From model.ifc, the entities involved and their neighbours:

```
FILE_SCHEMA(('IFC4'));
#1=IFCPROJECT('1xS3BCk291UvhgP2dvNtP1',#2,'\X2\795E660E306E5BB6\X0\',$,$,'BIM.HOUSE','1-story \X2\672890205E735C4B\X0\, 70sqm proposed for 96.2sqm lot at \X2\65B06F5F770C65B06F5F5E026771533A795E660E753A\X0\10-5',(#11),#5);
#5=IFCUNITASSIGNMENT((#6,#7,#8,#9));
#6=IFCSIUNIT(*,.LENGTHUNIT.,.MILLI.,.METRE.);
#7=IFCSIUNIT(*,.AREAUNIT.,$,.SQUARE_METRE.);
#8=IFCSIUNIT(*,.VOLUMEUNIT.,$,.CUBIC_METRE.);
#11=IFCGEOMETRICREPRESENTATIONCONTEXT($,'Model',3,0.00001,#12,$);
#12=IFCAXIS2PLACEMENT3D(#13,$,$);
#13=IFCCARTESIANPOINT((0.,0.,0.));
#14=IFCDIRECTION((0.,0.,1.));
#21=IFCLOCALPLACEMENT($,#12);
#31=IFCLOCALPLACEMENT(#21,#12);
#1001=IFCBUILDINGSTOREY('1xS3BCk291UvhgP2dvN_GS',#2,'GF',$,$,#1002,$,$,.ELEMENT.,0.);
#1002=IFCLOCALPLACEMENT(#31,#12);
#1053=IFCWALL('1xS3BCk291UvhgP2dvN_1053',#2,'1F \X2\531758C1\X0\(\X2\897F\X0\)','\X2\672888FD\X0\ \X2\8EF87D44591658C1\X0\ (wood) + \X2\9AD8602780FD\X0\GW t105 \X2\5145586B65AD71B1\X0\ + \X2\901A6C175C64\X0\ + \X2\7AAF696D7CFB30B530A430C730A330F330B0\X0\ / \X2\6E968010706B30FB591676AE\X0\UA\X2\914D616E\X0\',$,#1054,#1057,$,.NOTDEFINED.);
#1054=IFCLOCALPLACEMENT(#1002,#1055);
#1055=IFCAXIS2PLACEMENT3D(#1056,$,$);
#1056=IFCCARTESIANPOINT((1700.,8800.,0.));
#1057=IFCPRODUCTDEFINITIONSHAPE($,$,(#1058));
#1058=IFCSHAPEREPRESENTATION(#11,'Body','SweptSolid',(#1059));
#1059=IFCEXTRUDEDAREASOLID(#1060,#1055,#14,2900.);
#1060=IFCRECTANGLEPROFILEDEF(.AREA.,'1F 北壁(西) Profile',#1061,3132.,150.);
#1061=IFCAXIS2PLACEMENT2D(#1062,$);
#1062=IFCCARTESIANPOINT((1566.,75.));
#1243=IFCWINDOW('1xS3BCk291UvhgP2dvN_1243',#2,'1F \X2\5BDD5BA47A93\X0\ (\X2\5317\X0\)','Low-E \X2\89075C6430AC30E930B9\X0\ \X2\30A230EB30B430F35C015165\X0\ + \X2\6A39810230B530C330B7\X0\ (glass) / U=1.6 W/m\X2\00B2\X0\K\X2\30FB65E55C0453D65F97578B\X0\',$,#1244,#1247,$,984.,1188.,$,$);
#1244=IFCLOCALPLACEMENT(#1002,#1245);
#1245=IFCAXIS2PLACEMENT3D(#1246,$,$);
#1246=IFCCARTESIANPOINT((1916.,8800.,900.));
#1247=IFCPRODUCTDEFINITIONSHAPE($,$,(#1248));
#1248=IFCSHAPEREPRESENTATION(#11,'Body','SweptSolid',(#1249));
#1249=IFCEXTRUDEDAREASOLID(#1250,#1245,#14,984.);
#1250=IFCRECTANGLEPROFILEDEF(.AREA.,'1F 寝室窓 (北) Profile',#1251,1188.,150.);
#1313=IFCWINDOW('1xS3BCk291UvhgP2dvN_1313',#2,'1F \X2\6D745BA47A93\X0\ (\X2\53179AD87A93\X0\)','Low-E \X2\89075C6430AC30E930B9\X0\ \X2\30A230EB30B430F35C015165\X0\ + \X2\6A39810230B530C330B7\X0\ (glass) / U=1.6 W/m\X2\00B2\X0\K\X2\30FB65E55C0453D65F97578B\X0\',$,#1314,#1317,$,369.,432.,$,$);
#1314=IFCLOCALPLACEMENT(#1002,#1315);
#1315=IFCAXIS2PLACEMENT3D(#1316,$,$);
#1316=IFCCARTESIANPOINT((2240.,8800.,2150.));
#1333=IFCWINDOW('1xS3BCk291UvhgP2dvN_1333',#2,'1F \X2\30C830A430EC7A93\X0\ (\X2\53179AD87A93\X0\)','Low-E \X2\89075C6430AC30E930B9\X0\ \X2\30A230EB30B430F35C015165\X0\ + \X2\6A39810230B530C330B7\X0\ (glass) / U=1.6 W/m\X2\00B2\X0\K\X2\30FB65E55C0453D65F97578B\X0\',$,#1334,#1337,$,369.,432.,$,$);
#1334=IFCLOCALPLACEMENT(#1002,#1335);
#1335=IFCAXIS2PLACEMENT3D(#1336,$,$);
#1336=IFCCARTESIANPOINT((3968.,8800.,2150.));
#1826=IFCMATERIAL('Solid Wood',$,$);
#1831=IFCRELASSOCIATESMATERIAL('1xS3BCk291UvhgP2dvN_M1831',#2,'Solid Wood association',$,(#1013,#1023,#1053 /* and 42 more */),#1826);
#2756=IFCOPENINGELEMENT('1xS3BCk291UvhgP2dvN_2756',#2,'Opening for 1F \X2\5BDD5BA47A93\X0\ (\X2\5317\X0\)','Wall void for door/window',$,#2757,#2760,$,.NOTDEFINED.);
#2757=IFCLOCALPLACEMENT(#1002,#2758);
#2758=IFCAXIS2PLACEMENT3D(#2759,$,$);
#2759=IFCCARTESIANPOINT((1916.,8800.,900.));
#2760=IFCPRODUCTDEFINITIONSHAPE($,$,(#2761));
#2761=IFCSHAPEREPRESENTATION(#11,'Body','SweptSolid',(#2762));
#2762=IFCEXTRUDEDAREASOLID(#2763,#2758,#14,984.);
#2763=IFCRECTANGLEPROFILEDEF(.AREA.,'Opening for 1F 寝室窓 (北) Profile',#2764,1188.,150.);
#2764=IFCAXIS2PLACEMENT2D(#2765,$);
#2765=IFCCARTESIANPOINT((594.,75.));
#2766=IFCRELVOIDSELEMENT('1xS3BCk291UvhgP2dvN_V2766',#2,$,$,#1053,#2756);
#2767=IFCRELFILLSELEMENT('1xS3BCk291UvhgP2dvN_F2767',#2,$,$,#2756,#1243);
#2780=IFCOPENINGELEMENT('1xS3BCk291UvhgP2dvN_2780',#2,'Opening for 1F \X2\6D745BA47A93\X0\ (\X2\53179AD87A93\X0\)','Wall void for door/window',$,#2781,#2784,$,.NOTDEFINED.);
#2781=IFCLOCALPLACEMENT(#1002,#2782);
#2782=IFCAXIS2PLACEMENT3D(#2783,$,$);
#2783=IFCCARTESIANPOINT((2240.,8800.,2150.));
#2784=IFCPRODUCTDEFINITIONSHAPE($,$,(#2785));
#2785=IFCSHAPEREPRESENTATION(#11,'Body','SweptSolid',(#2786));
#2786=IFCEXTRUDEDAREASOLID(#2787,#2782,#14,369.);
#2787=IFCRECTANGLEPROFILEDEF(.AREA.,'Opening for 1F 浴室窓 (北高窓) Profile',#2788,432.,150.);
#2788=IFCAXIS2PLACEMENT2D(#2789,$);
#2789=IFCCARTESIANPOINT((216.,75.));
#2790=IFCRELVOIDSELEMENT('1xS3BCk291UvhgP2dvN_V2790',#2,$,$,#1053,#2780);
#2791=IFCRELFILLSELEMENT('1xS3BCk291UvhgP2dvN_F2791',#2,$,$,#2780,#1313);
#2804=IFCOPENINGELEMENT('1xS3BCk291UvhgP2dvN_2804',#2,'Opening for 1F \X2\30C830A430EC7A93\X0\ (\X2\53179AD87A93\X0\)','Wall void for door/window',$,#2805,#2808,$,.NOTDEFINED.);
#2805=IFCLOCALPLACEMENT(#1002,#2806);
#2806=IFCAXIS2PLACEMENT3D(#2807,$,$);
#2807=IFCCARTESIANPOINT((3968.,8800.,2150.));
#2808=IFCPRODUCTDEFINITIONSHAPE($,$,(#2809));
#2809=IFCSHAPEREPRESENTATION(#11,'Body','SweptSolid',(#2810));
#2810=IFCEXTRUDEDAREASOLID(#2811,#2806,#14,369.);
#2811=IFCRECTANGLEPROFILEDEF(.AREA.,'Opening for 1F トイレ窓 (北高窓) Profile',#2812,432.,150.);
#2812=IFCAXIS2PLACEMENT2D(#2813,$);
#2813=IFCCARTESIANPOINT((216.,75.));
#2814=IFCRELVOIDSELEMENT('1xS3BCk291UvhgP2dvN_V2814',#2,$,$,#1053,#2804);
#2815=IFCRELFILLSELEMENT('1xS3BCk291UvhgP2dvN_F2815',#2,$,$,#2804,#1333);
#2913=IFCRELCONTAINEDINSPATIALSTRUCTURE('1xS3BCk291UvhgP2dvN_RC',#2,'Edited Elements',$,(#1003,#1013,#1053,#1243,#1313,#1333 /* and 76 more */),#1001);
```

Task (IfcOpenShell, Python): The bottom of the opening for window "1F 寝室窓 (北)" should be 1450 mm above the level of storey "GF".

```python
import numpy as np
import ifcopenshell
import ifcopenshell.api.geometry
import ifcopenshell.geom
import ifcopenshell.util.element
import ifcopenshell.util.placement
import ifcopenshell.util.shape
import ifcopenshell.util.unit

model = ifcopenshell.open("model.ifc")
unit_scale = ifcopenshell.util.unit.calculate_unit_scale(model)

window = model.by_guid("1xS3BCk291UvhgP2dvN_1243")
opening = window.FillsVoids[0].RelatingOpeningElement
storey = ifcopenshell.util.element.get_container(window, ifc_class="IfcBuildingStorey")
level = ifcopenshell.util.placement.get_local_placement(storey.ObjectPlacement)[2, 3]

# The opening's origin need not be at the sill, so measure its lowest point.
shape = ifcopenshell.geom.create_shape(ifcopenshell.geom.settings(), opening)
bottom = ifcopenshell.util.shape.get_shape_bottom_elevation(shape, shape.geometry) / unit_scale
dz = level + 1.45 / unit_scale - bottom

shift = np.array([0.0, 0.0, dz])
# The window is not placed relative to its opening, so move both.
for product in (opening, window):
    matrix = ifcopenshell.util.placement.get_local_placement(product.ObjectPlacement)
    matrix[:3, 3] += shift
    ifcopenshell.api.geometry.edit_object_placement(model, product=product, matrix=matrix, is_si=False)

print(f"moved by {dz * unit_scale:+.3f} m")

model.write("model_rev.ifc")
```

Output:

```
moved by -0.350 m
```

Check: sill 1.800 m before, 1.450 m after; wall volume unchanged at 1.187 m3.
